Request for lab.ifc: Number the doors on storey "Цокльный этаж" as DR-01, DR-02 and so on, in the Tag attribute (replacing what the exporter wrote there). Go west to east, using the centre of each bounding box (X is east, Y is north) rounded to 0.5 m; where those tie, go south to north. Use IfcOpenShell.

First a look at what the model holds.

```python
import ifcopenshell
import ifcopenshell.util.element
import ifcopenshell.util.placement

model = ifcopenshell.open("lab.ifc")
print(model.schema)
storey = next(s for s in model.by_type("IfcBuildingStorey") if s.Name == "Цокльный этаж")
doors = [e for e in ifcopenshell.util.element.get_decomposition(storey) if e.is_a("IfcDoor")]
for e in sorted(doors, key=lambda e: e.id()):
    origin = ifcopenshell.util.placement.get_local_placement(e.ObjectPlacement)[:3, 3]
    print(e.id(), e.Tag, e.Name, origin.round(2) + 0.0, sep=" | ")
```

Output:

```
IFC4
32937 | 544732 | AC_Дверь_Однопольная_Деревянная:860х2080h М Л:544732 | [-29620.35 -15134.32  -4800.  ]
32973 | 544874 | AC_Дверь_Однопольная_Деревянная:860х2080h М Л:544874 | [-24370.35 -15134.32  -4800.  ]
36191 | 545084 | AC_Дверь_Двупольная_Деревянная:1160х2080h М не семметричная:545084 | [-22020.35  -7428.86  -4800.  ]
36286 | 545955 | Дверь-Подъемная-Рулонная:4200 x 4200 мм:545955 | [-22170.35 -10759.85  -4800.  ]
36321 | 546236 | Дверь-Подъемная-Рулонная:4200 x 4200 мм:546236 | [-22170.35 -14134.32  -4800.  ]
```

```python
import ifcopenshell
import ifcopenshell.geom
import ifcopenshell.util.element
import ifcopenshell.util.shape

model = ifcopenshell.open("lab.ifc")
settings = ifcopenshell.geom.settings()
settings.set("use-world-coords", True)


def centre(element):
    shape = ifcopenshell.geom.create_shape(settings, element)
    return ifcopenshell.util.shape.get_bbox_centroid(shape.geometry)


storey = next(s for s in model.by_type("IfcBuildingStorey") if s.Name == "Цокльный этаж")
doors = [e for e in ifcopenshell.util.element.get_decomposition(storey) if e.is_a("IfcDoor")]

# Insertion points can sit at a corner or the storey origin, so sort by the geometry (in metres).
centres = {e: centre(e) for e in doors}
doors.sort(key=lambda e: (round(centres[e][0] / 0.5), centres[e][1]))

for i, e in enumerate(doors, start=1):
    number = f"DR-{i:02d}"
    e.Tag = number
    print(e.id(), number)

model.write("lab_rev.ifc")
```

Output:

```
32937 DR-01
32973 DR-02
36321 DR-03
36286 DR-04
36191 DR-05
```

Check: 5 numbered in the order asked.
